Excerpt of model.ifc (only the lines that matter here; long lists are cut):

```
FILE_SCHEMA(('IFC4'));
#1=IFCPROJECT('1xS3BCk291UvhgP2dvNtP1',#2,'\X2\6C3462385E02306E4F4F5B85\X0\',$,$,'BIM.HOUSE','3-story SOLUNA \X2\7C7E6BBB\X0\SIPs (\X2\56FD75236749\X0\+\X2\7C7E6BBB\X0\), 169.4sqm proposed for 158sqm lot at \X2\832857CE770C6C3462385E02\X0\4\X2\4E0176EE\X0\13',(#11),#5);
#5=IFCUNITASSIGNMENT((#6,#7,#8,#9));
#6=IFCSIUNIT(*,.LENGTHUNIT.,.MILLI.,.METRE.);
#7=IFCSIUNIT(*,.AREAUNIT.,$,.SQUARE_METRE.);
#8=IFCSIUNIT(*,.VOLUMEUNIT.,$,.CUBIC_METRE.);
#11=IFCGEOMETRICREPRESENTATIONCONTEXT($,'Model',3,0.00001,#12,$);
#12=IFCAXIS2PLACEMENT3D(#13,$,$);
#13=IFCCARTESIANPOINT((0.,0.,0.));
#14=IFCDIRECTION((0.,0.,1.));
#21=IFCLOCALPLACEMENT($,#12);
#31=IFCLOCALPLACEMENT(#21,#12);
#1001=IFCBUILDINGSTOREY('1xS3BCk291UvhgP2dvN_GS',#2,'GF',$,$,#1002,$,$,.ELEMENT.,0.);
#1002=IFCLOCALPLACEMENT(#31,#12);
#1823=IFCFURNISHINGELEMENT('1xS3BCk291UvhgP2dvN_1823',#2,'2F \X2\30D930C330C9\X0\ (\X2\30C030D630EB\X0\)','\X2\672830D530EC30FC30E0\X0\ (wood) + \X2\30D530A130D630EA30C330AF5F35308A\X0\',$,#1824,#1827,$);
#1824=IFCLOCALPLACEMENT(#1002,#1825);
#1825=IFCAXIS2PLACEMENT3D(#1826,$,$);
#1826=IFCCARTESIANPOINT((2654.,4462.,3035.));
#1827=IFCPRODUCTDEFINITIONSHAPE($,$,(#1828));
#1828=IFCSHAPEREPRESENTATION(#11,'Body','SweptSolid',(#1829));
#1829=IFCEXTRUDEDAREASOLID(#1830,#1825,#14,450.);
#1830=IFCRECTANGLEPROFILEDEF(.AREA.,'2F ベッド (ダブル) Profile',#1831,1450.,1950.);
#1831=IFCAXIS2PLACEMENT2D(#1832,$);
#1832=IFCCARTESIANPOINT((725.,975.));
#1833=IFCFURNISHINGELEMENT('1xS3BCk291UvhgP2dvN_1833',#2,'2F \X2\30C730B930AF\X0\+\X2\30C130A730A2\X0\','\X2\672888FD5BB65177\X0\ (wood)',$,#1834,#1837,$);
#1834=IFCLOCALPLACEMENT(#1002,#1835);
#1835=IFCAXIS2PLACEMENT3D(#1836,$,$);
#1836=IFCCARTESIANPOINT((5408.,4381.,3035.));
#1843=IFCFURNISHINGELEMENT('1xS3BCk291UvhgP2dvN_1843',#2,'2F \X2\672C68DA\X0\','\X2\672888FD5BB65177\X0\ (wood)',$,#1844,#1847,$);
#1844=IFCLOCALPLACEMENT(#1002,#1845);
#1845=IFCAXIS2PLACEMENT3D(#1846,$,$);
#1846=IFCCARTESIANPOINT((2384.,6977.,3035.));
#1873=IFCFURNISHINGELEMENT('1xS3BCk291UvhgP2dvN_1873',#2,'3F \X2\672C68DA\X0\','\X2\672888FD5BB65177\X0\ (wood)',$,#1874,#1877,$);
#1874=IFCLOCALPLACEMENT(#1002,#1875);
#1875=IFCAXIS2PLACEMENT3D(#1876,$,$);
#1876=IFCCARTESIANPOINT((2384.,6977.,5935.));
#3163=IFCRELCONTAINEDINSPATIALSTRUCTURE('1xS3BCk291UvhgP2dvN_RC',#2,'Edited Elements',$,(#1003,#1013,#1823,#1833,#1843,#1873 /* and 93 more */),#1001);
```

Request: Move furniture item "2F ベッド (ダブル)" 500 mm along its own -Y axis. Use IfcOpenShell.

```python
import ifcopenshell
import ifcopenshell.api.geometry
import ifcopenshell.util.placement

model = ifcopenshell.open("model.ifc")

item = model.by_guid("1xS3BCk291UvhgP2dvN_1823")
matrix = ifcopenshell.util.placement.get_local_placement(item.ObjectPlacement)
matrix[:3, 3] -= matrix[:3, 1] * 500.0
ifcopenshell.api.geometry.edit_object_placement(model, product=item, matrix=matrix, is_si=False)

print(ifcopenshell.util.placement.get_local_placement(item.ObjectPlacement).round(3) + 0.0)

model.write("model-out.ifc")
```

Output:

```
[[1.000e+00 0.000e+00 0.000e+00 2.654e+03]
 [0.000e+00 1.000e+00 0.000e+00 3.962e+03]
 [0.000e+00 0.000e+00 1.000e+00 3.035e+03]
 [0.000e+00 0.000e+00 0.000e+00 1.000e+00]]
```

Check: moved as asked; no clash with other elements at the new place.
